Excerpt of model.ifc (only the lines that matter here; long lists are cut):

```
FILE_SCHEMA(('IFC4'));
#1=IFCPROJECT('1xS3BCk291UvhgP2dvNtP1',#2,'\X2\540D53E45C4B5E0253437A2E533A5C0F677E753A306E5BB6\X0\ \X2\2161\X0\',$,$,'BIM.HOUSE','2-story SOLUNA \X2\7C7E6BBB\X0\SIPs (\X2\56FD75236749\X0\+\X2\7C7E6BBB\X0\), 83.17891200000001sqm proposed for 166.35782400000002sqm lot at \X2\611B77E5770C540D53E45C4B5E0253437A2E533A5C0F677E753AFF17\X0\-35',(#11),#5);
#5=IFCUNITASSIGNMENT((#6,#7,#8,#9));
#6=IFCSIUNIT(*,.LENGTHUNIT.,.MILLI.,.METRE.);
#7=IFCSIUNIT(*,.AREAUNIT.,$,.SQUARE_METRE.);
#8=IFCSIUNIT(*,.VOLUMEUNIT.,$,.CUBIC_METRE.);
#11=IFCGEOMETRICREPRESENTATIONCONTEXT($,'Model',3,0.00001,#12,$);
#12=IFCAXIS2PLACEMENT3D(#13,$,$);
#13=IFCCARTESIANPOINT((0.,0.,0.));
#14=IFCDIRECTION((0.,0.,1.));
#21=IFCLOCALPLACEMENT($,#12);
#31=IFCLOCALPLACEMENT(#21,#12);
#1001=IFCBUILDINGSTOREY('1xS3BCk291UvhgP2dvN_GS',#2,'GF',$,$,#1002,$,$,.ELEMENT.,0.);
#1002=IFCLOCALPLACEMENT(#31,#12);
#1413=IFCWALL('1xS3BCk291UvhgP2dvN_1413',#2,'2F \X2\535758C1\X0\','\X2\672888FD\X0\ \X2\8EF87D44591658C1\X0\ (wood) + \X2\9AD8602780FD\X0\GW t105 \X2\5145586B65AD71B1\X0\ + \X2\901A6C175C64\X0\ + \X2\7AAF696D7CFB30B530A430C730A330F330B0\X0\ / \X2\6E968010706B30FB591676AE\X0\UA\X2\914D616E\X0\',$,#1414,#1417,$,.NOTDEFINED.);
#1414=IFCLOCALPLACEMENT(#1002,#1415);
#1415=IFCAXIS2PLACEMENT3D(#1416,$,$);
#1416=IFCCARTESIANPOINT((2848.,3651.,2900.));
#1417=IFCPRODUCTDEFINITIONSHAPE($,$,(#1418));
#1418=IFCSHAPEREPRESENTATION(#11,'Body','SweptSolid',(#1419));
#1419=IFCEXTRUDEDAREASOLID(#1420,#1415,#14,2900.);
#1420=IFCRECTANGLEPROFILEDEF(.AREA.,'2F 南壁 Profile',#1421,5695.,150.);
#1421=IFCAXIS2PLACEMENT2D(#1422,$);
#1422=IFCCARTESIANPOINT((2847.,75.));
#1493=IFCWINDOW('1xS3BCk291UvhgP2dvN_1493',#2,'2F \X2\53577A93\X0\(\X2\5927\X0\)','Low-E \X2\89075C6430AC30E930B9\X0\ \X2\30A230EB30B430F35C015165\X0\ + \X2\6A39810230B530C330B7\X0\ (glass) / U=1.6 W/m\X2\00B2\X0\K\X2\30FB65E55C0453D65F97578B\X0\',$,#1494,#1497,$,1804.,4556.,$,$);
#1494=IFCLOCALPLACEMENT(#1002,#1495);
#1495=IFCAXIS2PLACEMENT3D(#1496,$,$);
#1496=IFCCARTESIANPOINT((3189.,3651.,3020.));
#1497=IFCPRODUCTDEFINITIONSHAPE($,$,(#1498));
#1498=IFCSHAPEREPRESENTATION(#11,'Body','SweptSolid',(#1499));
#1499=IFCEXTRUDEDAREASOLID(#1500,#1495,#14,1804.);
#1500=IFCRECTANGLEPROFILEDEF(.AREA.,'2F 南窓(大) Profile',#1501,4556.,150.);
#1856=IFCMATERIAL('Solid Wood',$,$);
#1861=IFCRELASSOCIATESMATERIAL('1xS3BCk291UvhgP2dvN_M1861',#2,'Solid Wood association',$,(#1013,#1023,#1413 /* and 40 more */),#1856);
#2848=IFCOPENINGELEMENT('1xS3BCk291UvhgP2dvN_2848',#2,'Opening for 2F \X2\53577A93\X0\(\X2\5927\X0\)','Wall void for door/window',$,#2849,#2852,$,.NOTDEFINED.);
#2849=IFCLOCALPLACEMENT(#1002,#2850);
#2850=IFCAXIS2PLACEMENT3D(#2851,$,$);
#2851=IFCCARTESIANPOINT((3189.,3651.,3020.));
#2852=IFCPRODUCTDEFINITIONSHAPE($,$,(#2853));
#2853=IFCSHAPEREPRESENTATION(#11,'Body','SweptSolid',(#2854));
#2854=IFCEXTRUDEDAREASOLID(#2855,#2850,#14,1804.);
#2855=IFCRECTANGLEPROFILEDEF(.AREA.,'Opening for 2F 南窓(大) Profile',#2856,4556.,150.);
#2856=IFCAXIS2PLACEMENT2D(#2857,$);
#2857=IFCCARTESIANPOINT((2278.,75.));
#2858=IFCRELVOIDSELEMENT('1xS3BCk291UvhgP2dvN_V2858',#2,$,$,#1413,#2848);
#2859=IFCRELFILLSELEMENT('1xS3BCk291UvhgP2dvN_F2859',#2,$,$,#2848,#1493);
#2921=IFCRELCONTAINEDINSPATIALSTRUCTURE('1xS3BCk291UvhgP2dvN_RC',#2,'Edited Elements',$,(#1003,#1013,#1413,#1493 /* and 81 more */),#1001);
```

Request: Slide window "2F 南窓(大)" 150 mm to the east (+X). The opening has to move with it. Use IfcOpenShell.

```python
import ifcopenshell
import ifcopenshell.api.geometry
import ifcopenshell.util.placement
import ifcopenshell.util.unit

model = ifcopenshell.open("model.ifc")
unit_scale = ifcopenshell.util.unit.calculate_unit_scale(model)

window = model.by_guid("1xS3BCk291UvhgP2dvN_1493")
opening = window.FillsVoids[0].RelatingOpeningElement
wall = opening.VoidsElements[0].RelatingBuildingElement

wall_matrix = ifcopenshell.util.placement.get_local_placement(wall.ObjectPlacement)
shift = wall_matrix[:3, 0] * 0.15 / unit_scale
before = ifcopenshell.util.placement.get_local_placement(window.ObjectPlacement)[:3, 3].copy()

# The window is not placed relative to its opening, so move both.
for product in (opening, window):
    matrix = ifcopenshell.util.placement.get_local_placement(product.ObjectPlacement)
    matrix[:3, 3] += shift
    ifcopenshell.api.geometry.edit_object_placement(model, product=product, matrix=matrix, is_si=False)

after = ifcopenshell.util.placement.get_local_placement(window.ObjectPlacement)[:3, 3]
print("window moved by", (after - before).round(3) + 0.0)

model.write("model-out.ifc")
```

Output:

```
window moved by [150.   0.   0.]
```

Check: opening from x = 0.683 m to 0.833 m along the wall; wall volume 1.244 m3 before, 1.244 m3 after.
